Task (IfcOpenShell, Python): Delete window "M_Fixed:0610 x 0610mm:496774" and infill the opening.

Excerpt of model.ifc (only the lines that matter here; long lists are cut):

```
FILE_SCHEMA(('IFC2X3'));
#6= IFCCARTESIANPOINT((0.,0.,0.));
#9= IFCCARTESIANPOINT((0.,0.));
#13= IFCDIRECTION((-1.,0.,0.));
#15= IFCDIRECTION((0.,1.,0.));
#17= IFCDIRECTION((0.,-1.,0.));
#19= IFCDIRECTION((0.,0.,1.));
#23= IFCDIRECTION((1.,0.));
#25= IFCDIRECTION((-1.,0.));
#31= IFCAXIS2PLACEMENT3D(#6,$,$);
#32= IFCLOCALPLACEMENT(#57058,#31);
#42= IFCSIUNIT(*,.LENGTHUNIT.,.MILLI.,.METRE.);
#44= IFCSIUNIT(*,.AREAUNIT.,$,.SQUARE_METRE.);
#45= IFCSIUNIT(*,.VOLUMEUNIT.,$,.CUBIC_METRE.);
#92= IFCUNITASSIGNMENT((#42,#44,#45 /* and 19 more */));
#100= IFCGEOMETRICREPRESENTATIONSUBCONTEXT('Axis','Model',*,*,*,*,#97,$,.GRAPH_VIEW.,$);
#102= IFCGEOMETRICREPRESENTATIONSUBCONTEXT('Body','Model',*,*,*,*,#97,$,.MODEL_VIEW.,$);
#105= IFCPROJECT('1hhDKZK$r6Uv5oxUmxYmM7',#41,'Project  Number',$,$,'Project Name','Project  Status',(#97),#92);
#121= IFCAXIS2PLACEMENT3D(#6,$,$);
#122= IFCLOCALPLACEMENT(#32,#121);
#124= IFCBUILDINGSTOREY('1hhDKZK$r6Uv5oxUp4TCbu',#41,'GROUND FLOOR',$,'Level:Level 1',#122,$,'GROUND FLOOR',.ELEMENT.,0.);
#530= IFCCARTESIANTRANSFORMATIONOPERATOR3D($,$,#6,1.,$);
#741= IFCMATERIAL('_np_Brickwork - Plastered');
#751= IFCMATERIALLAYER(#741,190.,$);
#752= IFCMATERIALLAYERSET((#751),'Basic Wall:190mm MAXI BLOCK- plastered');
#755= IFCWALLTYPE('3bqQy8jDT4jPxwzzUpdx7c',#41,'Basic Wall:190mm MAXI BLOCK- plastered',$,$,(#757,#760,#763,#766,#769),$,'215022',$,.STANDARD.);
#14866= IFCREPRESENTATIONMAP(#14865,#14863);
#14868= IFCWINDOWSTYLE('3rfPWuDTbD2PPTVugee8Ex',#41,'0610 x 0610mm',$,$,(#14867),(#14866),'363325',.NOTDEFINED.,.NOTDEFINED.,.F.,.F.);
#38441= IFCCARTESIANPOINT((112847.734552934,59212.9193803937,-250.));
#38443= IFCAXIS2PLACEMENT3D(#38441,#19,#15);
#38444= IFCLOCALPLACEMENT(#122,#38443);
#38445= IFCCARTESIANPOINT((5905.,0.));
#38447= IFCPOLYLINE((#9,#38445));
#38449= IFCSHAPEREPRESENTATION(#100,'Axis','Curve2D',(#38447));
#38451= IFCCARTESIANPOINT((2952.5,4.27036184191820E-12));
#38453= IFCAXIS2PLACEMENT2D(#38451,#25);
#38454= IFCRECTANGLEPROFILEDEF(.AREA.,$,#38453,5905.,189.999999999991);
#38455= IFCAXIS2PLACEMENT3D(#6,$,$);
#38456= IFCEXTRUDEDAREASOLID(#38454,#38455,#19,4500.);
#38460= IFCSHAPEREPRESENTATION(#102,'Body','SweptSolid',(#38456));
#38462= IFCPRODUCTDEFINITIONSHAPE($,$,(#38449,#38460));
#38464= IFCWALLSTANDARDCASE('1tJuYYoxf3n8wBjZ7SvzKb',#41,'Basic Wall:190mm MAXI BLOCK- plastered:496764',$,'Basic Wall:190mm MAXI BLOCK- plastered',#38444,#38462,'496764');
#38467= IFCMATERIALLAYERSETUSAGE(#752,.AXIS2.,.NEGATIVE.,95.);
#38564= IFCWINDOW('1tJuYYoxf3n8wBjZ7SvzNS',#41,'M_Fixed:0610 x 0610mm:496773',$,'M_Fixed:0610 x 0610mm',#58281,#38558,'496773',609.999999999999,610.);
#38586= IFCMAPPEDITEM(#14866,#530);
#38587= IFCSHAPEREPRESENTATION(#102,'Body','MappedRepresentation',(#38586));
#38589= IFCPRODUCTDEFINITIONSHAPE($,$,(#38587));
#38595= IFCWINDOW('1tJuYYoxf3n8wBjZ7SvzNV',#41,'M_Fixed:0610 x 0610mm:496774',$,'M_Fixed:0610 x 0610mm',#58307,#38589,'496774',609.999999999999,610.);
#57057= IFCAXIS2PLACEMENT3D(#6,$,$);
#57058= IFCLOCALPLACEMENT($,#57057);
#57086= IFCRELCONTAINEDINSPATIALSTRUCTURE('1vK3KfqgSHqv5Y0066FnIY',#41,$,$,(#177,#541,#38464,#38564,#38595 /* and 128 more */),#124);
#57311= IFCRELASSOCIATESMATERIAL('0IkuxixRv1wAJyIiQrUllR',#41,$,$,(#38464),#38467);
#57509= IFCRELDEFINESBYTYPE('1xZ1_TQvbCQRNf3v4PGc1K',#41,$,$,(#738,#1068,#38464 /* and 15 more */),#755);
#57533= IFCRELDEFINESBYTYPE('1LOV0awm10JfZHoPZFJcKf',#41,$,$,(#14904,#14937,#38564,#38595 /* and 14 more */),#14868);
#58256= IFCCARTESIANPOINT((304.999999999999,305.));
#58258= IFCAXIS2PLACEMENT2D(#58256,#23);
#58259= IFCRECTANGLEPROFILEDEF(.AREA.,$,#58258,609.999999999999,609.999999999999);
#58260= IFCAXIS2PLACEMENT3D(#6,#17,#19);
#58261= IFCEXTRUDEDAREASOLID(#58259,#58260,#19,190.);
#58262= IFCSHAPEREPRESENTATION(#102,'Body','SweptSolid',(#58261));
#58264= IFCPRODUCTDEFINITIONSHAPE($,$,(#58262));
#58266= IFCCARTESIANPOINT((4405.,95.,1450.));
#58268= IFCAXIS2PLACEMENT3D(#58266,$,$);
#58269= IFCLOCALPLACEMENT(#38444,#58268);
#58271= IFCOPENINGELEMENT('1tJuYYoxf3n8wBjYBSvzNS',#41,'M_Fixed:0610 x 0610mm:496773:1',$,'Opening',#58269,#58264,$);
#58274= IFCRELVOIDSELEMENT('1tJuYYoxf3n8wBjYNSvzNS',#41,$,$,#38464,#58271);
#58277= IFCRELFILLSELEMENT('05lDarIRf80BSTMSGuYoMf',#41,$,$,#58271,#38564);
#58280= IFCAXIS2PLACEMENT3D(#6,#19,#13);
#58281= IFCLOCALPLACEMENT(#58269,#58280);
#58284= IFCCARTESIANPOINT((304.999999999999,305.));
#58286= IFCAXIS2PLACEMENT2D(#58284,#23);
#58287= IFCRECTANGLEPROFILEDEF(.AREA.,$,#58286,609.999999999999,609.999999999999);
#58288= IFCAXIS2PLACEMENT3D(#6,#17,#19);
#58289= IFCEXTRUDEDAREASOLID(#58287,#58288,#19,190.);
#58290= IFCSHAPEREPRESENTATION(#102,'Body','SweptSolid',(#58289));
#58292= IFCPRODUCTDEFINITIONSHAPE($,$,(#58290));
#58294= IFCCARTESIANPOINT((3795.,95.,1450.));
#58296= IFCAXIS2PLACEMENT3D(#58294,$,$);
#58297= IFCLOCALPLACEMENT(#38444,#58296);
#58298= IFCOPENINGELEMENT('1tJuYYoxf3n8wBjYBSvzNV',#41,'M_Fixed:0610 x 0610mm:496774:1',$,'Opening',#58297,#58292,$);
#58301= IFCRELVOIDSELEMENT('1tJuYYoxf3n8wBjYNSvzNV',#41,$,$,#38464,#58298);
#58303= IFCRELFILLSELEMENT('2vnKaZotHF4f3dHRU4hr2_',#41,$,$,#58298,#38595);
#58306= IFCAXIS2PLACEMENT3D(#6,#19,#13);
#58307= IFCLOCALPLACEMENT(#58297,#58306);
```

```python
import ifcopenshell
import ifcopenshell.api.feature
import ifcopenshell.api.root
import ifcopenshell.geom
import ifcopenshell.util.shape

model = ifcopenshell.open("model.ifc")
settings = ifcopenshell.geom.settings()


def volume(element):
    """Net volume in cubic metres, openings subtracted."""
    shape = ifcopenshell.geom.create_shape(settings, element)
    return ifcopenshell.util.shape.get_volume(shape.geometry)


window = model.by_id(38595)
opening = window.FillsVoids[0].RelatingOpeningElement
wall = opening.VoidsElements[0].RelatingBuildingElement
before = volume(wall)

ifcopenshell.api.root.remove_product(model, product=window)
ifcopenshell.api.feature.remove_feature(model, feature=opening)

after = volume(wall)

print(f"wall volume {before:.3f} -> {after:.3f} m3")

model.write("model_edited.ifc")
```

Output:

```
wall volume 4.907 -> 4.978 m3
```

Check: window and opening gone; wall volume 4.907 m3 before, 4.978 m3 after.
